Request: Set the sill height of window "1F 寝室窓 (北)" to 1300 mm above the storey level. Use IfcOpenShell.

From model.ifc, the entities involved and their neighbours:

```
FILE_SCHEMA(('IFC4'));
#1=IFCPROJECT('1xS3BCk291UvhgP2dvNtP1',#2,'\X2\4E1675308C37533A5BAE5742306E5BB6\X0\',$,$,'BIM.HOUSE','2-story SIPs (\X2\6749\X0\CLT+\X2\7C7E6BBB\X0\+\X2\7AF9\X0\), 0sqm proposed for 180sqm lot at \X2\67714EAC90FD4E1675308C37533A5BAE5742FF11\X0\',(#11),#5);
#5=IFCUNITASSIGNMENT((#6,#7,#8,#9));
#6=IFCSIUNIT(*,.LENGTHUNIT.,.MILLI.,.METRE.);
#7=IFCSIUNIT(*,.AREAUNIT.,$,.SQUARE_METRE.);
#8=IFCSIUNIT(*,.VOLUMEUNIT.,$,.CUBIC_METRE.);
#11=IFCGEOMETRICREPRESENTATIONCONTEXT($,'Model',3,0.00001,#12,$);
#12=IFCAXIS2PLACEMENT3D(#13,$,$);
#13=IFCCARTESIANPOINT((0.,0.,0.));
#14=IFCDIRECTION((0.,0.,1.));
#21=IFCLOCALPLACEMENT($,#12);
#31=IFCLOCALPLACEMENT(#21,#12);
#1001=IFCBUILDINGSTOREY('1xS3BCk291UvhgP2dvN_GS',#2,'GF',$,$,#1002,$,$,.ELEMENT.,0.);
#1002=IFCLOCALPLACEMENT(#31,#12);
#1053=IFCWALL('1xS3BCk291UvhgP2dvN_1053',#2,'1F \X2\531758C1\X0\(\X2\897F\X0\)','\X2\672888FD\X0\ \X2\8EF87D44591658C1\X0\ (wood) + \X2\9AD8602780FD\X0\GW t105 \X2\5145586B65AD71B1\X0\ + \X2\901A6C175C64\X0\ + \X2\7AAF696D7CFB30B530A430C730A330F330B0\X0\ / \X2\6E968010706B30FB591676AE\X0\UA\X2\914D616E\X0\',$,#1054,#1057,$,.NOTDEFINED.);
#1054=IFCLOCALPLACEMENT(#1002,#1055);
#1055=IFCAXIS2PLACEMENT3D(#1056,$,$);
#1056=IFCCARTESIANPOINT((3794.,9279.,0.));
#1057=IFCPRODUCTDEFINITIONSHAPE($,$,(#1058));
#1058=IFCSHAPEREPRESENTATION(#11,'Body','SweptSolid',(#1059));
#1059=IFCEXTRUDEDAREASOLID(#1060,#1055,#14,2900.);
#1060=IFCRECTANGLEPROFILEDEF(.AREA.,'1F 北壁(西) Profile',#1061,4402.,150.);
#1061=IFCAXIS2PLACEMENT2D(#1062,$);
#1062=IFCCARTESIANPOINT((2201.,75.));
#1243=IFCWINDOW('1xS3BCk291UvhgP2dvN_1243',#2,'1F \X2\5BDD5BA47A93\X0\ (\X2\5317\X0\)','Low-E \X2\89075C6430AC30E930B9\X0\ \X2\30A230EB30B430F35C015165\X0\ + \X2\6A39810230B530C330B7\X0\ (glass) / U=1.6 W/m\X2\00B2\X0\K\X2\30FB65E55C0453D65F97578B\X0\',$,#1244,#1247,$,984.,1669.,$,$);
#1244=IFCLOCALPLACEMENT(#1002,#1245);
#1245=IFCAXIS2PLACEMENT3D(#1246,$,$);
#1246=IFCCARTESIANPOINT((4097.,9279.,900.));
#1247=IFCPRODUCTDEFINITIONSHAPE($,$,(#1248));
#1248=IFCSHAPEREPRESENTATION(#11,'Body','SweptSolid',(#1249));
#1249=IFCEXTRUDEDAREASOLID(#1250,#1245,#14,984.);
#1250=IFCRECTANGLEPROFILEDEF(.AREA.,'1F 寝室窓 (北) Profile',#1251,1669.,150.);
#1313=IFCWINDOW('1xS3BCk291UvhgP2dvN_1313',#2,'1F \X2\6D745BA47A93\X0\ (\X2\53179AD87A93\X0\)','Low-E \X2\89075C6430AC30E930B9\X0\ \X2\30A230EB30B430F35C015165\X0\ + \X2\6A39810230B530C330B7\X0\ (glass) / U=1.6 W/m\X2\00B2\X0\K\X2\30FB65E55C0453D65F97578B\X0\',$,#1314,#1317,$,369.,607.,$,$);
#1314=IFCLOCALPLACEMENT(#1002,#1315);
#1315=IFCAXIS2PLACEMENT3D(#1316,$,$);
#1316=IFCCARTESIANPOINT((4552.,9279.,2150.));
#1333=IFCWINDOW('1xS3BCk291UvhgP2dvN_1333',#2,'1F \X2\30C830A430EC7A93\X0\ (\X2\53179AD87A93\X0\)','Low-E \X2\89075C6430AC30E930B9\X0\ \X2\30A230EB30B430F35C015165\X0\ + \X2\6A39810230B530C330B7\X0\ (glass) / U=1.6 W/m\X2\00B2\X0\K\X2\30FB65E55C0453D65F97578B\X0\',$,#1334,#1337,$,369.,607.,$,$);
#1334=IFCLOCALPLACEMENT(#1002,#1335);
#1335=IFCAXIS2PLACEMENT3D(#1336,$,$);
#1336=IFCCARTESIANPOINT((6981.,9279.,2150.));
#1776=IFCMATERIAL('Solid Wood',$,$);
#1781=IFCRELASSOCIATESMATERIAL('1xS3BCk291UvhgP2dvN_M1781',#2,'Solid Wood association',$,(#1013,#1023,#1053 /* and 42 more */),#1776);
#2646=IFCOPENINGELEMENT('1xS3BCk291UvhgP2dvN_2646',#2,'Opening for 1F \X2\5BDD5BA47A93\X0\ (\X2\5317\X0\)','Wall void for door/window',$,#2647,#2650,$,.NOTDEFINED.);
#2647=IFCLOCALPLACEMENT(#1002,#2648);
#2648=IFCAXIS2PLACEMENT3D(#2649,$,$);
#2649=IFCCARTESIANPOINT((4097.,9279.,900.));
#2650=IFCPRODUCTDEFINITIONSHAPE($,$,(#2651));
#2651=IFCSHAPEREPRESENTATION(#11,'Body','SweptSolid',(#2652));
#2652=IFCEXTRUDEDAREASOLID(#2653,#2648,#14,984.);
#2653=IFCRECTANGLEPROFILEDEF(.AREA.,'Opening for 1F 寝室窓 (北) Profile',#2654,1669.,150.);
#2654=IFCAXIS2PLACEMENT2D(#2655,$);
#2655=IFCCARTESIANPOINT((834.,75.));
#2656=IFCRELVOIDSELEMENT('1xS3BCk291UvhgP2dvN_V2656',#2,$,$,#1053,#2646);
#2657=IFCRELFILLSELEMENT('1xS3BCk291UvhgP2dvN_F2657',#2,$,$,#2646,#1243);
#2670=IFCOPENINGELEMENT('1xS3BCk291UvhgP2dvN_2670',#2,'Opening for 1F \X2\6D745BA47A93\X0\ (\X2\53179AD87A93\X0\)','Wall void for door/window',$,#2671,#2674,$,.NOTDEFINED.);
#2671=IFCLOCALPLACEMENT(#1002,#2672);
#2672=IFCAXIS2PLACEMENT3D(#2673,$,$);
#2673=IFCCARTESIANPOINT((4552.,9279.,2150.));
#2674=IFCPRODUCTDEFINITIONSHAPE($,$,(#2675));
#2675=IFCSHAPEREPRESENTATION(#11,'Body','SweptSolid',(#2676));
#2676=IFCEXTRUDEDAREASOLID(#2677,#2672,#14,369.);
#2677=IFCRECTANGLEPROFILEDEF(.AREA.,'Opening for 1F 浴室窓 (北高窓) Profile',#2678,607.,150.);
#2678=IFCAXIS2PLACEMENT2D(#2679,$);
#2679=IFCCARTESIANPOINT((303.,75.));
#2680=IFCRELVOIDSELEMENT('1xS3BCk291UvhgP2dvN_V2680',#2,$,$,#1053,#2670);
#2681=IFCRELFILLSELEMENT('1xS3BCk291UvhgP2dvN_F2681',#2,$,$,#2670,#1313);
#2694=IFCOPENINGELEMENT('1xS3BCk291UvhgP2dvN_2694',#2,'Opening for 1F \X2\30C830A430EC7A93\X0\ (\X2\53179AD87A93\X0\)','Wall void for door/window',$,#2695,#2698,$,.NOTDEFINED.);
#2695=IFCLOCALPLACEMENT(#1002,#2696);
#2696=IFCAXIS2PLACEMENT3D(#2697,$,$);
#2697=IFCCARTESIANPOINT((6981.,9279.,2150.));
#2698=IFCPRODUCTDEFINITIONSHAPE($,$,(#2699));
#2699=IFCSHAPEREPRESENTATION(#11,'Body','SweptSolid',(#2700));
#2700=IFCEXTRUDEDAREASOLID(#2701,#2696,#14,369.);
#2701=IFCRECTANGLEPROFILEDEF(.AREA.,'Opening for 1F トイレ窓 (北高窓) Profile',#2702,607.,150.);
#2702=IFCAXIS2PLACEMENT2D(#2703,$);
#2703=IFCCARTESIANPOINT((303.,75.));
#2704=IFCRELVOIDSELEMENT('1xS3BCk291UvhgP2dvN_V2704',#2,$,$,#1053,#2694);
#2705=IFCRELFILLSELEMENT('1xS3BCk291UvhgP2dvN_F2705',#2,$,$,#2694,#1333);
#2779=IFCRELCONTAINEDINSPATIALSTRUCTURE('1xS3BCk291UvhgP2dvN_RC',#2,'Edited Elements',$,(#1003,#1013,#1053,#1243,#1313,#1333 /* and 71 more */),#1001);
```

```python
import numpy as np
import ifcopenshell
import ifcopenshell.api.geometry
import ifcopenshell.geom
import ifcopenshell.util.element
import ifcopenshell.util.placement
import ifcopenshell.util.shape
import ifcopenshell.util.unit

model = ifcopenshell.open("model.ifc")
unit_scale = ifcopenshell.util.unit.calculate_unit_scale(model)

window = model.by_id(1243)
opening = window.FillsVoids[0].RelatingOpeningElement
storey = ifcopenshell.util.element.get_container(window, ifc_class="IfcBuildingStorey")
level = ifcopenshell.util.placement.get_local_placement(storey.ObjectPlacement)[2, 3]

# The opening's origin need not be at the sill, so measure its lowest point.
shape = ifcopenshell.geom.create_shape(ifcopenshell.geom.settings(), opening)
bottom = ifcopenshell.util.shape.get_shape_bottom_elevation(shape, shape.geometry) / unit_scale
dz = level + 1.3 / unit_scale - bottom

shift = np.array([0.0, 0.0, dz])
# The window is not placed relative to its opening, so move both.
for product in (opening, window):
    matrix = ifcopenshell.util.placement.get_local_placement(product.ObjectPlacement)
    matrix[:3, 3] += shift
    ifcopenshell.api.geometry.edit_object_placement(model, product=product, matrix=matrix, is_si=False)

print(f"moved by {dz * unit_scale:+.3f} m")

model.write("model_rev.ifc")
```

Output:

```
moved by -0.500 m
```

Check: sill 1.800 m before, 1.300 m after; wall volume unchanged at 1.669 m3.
